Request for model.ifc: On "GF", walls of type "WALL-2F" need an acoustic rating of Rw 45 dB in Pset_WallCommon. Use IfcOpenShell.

First a look at what the model holds.

```python
import ifcopenshell
import ifcopenshell.util.element

model = ifcopenshell.open("model.ifc")
print(model.schema)
storey = next(s for s in model.by_type("IfcBuildingStorey") if s.Name == "GF")
walls = [e for e in ifcopenshell.util.element.get_decomposition(storey) if e.is_a("IfcWall")]
seen = {}
for e in walls:
    element_type = ifcopenshell.util.element.get_type(e)
    key = (element_type.Name if element_type != e and element_type else None, ifcopenshell.util.element.get_pset(e, "Pset_WallCommon", "AcousticRating"))
    seen[key] = seen.get(key, 0) + 1
for (name, value), count in sorted(seen.items(), key=str):
    print(count, "x", name, "|", value)
```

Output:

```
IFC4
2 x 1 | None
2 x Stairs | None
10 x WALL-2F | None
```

```python
import ifcopenshell
import ifcopenshell.api.pset
import ifcopenshell.util.element

model = ifcopenshell.open("model.ifc")

storey = next(s for s in model.by_type("IfcBuildingStorey") if s.Name == "GF")
walls = [e for e in ifcopenshell.util.element.get_decomposition(storey) if e.is_a("IfcWall")]

count = 0
for e in walls:
    element_type = ifcopenshell.util.element.get_type(e)
    if element_type in (None, e) or element_type.Name != "WALL-2F":
        continue
    # add_pset returns the element's existing set when there is one.
    pset = ifcopenshell.api.pset.add_pset(model, product=e, name="Pset_WallCommon")
    ifcopenshell.api.pset.edit_pset(model, pset=pset, properties={"AcousticRating": "Rw 45 dB"})
    count += 1

print(count, "walls updated")

model.write("model_v2.ifc")
```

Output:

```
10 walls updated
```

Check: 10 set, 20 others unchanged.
